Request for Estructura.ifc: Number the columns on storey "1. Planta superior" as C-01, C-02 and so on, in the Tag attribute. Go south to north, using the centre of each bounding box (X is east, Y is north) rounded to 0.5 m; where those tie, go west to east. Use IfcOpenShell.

First a look at what the model holds.

```python
import ifcopenshell
import ifcopenshell.util.element
import ifcopenshell.util.placement

model = ifcopenshell.open("Estructura.ifc")
print(model.schema)
storey = next(s for s in model.by_type("IfcBuildingStorey") if s.Name == "1. Planta superior")
columns = [e for e in ifcopenshell.util.element.get_decomposition(storey) if e.is_a("IfcColumn")]
for e in sorted(columns, key=lambda e: e.id()):
    origin = ifcopenshell.util.placement.get_local_placement(e.ObjectPlacement)[:3, 3]
    print(e.id(), e.Tag, e.Name, origin.round(2) + 0.0, sep=" | ")
```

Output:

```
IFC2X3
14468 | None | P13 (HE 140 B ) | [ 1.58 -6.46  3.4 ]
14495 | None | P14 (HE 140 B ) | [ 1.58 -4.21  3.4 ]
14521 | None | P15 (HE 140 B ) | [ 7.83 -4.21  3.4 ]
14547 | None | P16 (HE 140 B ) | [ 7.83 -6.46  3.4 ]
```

```python
import ifcopenshell
import ifcopenshell.geom
import ifcopenshell.util.element
import ifcopenshell.util.shape

model = ifcopenshell.open("Estructura.ifc")
settings = ifcopenshell.geom.settings()
settings.set("use-world-coords", True)


def centre(element):
    shape = ifcopenshell.geom.create_shape(settings, element)
    return ifcopenshell.util.shape.get_bbox_centroid(shape.geometry)


storey = next(s for s in model.by_type("IfcBuildingStorey") if s.Name == "1. Planta superior")
columns = [e for e in ifcopenshell.util.element.get_decomposition(storey) if e.is_a("IfcColumn")]

# Insertion points can sit at a corner or the storey origin, so sort by the geometry (in metres).
centres = {e: centre(e) for e in columns}
columns.sort(key=lambda e: (round(centres[e][1] / 0.5), centres[e][0]))

for i, e in enumerate(columns, start=1):
    number = f"C-{i:02d}"
    e.Tag = number
    print(e.id(), number)

model.write("Estructura_edited.ifc")
```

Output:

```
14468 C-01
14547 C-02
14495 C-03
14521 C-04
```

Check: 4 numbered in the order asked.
